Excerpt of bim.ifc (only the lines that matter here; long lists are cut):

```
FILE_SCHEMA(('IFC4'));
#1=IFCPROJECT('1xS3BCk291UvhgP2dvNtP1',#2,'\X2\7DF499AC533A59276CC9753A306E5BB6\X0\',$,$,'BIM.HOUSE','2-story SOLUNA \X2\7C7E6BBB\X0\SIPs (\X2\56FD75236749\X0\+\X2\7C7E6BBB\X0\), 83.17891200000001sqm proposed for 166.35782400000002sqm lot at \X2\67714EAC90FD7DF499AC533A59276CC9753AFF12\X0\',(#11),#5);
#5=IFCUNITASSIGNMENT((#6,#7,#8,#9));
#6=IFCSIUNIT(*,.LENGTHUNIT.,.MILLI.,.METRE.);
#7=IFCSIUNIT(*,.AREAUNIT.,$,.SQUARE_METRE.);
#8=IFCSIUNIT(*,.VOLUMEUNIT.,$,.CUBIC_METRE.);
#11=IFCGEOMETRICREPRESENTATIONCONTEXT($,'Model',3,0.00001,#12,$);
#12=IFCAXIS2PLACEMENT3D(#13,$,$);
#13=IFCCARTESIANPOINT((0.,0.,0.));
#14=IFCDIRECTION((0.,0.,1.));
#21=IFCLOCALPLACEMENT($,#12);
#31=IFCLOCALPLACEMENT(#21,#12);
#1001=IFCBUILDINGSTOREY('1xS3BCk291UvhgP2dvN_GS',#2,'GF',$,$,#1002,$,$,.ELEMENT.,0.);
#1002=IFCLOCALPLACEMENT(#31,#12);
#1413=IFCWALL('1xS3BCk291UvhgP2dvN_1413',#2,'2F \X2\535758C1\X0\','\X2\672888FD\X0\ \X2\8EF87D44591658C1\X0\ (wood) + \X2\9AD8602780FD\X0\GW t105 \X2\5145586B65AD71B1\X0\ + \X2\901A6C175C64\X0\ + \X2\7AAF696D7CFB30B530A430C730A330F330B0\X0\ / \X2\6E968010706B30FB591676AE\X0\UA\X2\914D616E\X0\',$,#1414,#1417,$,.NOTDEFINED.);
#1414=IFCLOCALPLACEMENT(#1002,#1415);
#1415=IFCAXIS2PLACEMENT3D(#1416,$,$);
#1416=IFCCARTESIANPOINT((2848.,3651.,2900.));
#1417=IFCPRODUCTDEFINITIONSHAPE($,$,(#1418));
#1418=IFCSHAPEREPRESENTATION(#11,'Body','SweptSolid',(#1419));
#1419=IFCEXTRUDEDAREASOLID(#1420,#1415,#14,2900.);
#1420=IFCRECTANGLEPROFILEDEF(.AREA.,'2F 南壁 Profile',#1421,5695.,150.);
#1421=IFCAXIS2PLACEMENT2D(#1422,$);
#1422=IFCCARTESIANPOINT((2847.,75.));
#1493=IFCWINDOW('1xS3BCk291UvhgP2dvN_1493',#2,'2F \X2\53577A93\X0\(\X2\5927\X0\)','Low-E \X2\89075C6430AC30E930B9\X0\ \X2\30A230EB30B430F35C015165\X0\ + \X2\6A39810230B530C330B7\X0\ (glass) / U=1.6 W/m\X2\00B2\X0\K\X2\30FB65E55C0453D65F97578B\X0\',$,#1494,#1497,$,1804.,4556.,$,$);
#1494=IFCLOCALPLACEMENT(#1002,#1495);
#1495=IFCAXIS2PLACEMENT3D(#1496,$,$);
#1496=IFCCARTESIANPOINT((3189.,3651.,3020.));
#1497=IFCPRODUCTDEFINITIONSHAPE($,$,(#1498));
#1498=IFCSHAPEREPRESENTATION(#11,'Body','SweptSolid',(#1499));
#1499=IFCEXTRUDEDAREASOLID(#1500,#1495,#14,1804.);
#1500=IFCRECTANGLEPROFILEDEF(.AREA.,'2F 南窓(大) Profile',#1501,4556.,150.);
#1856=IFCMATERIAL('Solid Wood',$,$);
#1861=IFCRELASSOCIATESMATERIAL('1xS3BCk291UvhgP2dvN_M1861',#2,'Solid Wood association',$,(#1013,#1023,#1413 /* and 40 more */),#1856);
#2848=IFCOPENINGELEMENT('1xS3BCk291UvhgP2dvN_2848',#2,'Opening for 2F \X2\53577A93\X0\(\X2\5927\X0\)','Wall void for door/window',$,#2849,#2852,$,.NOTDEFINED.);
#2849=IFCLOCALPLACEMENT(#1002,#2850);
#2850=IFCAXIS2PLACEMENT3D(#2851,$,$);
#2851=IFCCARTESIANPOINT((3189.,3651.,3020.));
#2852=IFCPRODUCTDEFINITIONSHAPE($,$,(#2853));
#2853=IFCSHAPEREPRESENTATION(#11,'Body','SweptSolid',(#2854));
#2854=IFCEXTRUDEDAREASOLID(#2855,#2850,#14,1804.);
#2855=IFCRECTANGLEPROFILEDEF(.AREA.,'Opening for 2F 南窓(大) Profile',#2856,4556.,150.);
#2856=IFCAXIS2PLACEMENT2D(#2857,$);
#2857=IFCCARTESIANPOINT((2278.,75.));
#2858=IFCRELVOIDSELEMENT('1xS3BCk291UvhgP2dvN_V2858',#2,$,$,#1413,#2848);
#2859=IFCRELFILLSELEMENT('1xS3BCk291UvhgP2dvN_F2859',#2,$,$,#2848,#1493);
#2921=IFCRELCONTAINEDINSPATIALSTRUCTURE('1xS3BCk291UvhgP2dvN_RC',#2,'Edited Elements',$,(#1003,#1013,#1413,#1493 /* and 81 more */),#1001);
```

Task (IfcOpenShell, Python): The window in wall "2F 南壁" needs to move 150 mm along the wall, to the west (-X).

```python
import ifcopenshell
import ifcopenshell.api.geometry
import ifcopenshell.util.placement
import ifcopenshell.util.unit

model = ifcopenshell.open("bim.ifc")
unit_scale = ifcopenshell.util.unit.calculate_unit_scale(model)

window = model.by_guid("1xS3BCk291UvhgP2dvN_1493")
opening = window.FillsVoids[0].RelatingOpeningElement
wall = opening.VoidsElements[0].RelatingBuildingElement

wall_matrix = ifcopenshell.util.placement.get_local_placement(wall.ObjectPlacement)
shift = wall_matrix[:3, 0] * -0.15 / unit_scale
before = ifcopenshell.util.placement.get_local_placement(window.ObjectPlacement)[:3, 3].copy()

# The window is not placed relative to its opening, so move both.
for product in (opening, window):
    matrix = ifcopenshell.util.placement.get_local_placement(product.ObjectPlacement)
    matrix[:3, 3] += shift
    ifcopenshell.api.geometry.edit_object_placement(model, product=product, matrix=matrix, is_si=False)

after = ifcopenshell.util.placement.get_local_placement(window.ObjectPlacement)[:3, 3]
print("window moved by", (after - before).round(3) + 0.0)

model.write("bim_v2.ifc")
```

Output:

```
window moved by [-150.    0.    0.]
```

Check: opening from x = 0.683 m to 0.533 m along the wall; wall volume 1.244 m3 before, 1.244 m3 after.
